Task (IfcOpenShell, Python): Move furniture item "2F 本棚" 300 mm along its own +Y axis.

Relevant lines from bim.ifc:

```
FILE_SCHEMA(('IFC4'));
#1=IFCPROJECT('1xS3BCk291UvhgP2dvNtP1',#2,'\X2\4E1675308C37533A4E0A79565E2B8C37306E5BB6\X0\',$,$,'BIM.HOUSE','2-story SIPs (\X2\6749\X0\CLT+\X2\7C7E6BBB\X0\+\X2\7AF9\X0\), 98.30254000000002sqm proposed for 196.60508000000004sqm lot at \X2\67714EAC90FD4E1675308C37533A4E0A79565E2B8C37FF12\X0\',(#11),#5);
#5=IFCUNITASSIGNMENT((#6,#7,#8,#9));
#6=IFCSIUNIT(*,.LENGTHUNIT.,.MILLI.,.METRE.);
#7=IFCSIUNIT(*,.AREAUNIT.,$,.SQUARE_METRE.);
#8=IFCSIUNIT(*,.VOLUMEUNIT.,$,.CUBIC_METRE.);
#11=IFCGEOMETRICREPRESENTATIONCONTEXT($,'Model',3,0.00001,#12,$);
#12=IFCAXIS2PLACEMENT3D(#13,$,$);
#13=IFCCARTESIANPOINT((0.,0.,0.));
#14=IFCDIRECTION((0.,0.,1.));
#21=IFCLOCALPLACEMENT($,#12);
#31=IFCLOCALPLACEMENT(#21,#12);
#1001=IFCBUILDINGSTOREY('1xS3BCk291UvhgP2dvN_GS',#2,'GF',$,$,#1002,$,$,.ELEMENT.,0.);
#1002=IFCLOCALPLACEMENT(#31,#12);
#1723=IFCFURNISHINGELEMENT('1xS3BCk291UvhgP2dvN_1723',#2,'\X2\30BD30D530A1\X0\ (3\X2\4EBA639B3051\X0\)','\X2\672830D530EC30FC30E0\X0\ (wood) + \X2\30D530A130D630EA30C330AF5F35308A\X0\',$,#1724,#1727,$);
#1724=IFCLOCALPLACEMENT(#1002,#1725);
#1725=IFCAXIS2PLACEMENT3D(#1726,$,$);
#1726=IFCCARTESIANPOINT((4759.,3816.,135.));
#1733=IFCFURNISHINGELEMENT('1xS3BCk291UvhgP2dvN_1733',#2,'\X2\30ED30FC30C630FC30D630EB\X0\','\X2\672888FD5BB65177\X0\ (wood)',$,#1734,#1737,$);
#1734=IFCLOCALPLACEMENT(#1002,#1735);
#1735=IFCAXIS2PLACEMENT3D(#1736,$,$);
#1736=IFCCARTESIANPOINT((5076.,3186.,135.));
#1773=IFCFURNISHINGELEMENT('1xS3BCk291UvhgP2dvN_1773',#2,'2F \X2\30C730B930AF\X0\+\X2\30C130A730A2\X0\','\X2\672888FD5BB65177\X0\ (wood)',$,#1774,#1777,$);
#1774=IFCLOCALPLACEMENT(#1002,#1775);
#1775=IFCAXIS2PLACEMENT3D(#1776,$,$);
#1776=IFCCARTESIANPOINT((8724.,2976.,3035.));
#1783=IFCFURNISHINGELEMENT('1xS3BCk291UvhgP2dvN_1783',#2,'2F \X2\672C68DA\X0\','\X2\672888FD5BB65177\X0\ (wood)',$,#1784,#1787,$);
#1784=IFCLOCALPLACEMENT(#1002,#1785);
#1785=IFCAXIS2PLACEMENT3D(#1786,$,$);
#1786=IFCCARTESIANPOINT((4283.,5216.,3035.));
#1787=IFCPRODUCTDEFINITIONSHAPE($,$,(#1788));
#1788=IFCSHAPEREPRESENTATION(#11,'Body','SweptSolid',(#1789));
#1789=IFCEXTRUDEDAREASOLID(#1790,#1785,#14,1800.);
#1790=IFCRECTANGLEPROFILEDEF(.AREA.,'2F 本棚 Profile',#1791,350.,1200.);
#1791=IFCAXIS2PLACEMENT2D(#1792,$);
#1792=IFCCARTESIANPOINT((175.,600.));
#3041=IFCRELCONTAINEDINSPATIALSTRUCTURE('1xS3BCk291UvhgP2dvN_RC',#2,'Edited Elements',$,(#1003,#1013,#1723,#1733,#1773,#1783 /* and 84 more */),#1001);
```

```python
import ifcopenshell
import ifcopenshell.api.geometry
import ifcopenshell.util.placement

model = ifcopenshell.open("bim.ifc")

item = model.by_guid("1xS3BCk291UvhgP2dvN_1783")
matrix = ifcopenshell.util.placement.get_local_placement(item.ObjectPlacement)
matrix[:3, 3] += matrix[:3, 1] * 300.0
ifcopenshell.api.geometry.edit_object_placement(model, product=item, matrix=matrix, is_si=False)

print(ifcopenshell.util.placement.get_local_placement(item.ObjectPlacement).round(3) + 0.0)

model.write("bim-out.ifc")
```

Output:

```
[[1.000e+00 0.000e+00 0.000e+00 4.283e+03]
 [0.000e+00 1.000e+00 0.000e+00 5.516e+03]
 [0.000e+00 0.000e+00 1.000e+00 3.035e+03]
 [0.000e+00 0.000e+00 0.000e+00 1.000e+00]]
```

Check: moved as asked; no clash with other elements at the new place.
